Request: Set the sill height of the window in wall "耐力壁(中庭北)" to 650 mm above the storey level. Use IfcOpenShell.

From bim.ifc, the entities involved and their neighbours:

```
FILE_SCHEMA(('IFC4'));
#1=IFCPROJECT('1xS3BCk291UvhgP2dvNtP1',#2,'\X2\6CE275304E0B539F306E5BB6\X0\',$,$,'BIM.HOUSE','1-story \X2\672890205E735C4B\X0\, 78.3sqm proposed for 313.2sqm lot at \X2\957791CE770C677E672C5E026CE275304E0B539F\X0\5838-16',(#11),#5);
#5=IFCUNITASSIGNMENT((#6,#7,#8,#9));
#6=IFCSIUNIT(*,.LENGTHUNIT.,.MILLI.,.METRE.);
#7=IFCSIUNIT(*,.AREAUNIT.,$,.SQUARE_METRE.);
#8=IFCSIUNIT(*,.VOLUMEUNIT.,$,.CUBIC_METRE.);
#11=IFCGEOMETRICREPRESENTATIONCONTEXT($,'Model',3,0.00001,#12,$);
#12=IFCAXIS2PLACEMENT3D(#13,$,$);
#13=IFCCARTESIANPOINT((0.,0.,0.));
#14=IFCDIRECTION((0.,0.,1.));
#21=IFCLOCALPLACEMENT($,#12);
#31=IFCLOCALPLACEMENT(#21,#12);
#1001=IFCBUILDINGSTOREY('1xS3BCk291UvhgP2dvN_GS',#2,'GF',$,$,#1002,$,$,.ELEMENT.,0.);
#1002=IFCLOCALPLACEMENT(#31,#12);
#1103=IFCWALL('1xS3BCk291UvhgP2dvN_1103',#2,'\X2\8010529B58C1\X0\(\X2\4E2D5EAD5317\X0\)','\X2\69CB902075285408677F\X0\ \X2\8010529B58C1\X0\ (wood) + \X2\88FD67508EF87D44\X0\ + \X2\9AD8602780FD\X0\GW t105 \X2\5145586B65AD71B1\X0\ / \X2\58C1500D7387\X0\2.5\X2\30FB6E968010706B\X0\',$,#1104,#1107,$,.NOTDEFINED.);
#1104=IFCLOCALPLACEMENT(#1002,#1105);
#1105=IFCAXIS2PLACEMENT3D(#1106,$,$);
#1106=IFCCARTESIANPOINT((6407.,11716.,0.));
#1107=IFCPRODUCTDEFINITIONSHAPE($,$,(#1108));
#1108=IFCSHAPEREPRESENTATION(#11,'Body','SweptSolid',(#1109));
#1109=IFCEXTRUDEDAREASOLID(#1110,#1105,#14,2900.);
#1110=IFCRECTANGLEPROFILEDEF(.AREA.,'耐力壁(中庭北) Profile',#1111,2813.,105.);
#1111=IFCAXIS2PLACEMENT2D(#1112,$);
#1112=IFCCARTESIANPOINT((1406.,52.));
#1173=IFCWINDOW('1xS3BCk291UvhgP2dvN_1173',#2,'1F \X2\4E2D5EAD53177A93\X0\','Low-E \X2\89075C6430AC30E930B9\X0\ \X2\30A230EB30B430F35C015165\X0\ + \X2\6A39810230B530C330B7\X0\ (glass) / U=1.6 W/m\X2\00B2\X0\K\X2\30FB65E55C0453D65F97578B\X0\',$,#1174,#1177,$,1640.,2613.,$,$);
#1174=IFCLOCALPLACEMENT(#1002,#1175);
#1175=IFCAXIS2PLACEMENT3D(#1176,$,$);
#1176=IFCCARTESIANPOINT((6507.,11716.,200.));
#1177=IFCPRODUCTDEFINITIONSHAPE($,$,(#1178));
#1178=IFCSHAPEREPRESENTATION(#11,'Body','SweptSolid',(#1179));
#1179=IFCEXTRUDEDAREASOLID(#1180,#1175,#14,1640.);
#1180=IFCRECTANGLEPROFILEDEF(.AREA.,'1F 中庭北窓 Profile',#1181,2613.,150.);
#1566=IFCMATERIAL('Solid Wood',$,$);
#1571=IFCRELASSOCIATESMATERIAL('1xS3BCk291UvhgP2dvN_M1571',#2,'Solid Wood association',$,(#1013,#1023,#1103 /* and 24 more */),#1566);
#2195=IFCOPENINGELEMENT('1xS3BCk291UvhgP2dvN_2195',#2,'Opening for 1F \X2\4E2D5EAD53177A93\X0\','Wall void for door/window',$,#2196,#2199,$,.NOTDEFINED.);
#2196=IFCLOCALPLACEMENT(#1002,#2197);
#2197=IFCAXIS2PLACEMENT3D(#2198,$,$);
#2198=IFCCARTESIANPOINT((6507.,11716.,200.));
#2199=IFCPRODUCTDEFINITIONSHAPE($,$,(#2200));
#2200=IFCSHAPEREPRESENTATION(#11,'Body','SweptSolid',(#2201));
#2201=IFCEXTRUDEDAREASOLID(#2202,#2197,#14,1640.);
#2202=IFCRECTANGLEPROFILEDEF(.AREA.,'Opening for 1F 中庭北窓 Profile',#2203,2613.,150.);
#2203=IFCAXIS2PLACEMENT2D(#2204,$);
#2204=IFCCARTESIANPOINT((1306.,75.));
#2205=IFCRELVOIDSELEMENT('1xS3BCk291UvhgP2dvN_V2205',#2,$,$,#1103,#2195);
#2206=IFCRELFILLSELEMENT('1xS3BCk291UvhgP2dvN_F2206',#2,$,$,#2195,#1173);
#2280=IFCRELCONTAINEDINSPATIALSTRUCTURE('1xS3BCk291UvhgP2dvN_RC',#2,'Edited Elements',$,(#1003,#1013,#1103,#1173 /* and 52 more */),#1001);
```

```python
import numpy as np
import ifcopenshell
import ifcopenshell.api.geometry
import ifcopenshell.geom
import ifcopenshell.util.element
import ifcopenshell.util.placement
import ifcopenshell.util.shape
import ifcopenshell.util.unit

model = ifcopenshell.open("bim.ifc")
unit_scale = ifcopenshell.util.unit.calculate_unit_scale(model)

window = model.by_guid("1xS3BCk291UvhgP2dvN_1173")
opening = window.FillsVoids[0].RelatingOpeningElement
storey = ifcopenshell.util.element.get_container(window, ifc_class="IfcBuildingStorey")
level = ifcopenshell.util.placement.get_local_placement(storey.ObjectPlacement)[2, 3]

# The opening's origin need not be at the sill, so measure its lowest point.
shape = ifcopenshell.geom.create_shape(ifcopenshell.geom.settings(), opening)
bottom = ifcopenshell.util.shape.get_shape_bottom_elevation(shape, shape.geometry) / unit_scale
dz = level + 650.0 - bottom

shift = np.array([0.0, 0.0, dz])
# The window is not placed relative to its opening, so move both.
for product in (opening, window):
    matrix = ifcopenshell.util.placement.get_local_placement(product.ObjectPlacement)
    matrix[:3, 3] += shift
    ifcopenshell.api.geometry.edit_object_placement(model, product=product, matrix=matrix, is_si=False)

print(f"moved by {dz * unit_scale:+.3f} m")

model.write("bim_v2.ifc")
```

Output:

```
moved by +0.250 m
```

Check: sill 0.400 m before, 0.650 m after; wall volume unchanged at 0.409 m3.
